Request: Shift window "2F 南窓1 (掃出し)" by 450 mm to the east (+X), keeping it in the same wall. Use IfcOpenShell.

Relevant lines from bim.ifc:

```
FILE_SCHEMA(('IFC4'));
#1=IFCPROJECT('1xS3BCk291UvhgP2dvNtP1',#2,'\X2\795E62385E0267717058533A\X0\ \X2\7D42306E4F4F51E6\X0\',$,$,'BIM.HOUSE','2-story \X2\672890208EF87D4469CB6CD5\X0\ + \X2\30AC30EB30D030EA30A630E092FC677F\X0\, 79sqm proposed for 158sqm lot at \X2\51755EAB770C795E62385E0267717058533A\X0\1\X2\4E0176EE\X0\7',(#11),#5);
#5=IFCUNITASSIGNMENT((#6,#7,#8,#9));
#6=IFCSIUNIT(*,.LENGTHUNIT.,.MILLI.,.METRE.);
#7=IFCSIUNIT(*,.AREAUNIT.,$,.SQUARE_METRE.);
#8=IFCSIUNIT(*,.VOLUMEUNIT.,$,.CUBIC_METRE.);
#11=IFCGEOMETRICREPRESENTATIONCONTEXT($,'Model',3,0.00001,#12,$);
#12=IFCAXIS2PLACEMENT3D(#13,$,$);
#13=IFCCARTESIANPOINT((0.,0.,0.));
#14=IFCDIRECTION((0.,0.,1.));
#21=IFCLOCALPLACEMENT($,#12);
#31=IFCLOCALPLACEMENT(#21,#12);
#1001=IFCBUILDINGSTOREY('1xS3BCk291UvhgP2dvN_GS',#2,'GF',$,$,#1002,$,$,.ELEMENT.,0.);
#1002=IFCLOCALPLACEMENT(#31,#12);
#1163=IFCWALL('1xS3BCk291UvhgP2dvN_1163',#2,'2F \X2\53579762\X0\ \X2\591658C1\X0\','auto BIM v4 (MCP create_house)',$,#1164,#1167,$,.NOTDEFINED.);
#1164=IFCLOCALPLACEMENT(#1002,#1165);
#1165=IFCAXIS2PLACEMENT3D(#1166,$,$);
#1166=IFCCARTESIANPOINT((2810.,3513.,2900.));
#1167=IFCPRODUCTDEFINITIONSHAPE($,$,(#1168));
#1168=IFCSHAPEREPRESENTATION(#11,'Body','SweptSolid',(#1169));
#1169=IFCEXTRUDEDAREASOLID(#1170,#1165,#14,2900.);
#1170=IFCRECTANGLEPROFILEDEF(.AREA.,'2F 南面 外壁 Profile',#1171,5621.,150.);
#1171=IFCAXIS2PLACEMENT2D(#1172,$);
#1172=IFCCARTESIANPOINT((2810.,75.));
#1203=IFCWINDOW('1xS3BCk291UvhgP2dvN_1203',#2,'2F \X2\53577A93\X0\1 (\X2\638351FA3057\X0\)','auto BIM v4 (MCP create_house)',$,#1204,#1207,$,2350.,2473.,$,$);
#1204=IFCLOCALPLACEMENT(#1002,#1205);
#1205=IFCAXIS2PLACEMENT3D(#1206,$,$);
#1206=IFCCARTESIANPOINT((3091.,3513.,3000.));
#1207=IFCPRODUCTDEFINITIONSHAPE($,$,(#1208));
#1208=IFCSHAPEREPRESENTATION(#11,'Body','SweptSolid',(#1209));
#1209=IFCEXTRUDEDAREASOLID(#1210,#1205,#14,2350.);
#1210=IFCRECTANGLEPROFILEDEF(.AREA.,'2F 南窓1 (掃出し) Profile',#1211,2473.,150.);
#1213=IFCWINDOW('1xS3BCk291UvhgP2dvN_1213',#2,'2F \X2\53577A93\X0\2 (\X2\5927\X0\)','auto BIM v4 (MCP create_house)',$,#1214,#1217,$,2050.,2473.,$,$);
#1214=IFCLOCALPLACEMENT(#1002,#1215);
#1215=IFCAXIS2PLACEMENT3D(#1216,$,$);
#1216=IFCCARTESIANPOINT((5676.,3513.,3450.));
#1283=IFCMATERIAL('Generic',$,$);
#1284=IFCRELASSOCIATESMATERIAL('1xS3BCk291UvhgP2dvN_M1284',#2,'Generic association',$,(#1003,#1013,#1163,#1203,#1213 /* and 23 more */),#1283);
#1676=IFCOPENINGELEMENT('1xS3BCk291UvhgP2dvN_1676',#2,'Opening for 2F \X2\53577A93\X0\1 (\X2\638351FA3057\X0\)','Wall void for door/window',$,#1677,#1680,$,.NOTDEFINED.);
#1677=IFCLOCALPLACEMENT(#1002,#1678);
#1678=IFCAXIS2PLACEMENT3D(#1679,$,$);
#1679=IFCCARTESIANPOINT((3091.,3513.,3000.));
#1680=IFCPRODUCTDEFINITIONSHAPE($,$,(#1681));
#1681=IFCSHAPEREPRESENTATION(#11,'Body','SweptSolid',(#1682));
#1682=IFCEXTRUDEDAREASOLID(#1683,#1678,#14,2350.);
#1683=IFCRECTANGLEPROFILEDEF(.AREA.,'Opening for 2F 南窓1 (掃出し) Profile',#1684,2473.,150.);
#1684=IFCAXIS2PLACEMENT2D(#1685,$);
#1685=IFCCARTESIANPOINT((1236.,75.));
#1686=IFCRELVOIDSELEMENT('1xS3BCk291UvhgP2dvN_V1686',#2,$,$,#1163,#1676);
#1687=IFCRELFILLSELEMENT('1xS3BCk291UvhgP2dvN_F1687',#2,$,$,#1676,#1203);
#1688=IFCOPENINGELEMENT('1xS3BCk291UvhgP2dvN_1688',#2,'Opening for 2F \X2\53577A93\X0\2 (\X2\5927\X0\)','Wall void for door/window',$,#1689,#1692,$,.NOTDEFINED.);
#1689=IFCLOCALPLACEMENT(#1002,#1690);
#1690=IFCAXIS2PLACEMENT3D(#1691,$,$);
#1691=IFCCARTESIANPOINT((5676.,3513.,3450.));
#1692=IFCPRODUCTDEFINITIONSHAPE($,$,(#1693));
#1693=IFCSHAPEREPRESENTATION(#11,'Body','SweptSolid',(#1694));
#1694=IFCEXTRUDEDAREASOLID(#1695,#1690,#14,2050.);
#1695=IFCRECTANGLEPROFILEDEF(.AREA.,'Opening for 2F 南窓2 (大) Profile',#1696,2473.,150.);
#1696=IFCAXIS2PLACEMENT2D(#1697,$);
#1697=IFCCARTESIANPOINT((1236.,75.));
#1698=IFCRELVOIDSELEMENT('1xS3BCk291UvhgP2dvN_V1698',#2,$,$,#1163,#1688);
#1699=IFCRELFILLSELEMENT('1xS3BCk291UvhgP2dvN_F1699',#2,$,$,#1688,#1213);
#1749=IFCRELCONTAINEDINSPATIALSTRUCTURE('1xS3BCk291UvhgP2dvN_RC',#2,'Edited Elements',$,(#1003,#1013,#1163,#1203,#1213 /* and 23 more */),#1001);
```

```python
import ifcopenshell
import ifcopenshell.api.geometry
import ifcopenshell.util.placement
import ifcopenshell.util.unit

model = ifcopenshell.open("bim.ifc")
unit_scale = ifcopenshell.util.unit.calculate_unit_scale(model)

window = model.by_guid("1xS3BCk291UvhgP2dvN_1203")
opening = window.FillsVoids[0].RelatingOpeningElement
wall = opening.VoidsElements[0].RelatingBuildingElement

wall_matrix = ifcopenshell.util.placement.get_local_placement(wall.ObjectPlacement)
shift = wall_matrix[:3, 0] * 0.45 / unit_scale
before = ifcopenshell.util.placement.get_local_placement(window.ObjectPlacement)[:3, 3].copy()

# The window is not placed relative to its opening, so move both.
for product in (opening, window):
    matrix = ifcopenshell.util.placement.get_local_placement(product.ObjectPlacement)
    matrix[:3, 3] += shift
    ifcopenshell.api.geometry.edit_object_placement(model, product=product, matrix=matrix, is_si=False)

after = ifcopenshell.util.placement.get_local_placement(window.ObjectPlacement)[:3, 3]
print("window moved by", (after - before).round(3) + 0.0)

model.write("bim_edited.ifc")
```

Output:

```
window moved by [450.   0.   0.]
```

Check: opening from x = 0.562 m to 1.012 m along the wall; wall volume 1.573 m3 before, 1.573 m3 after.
